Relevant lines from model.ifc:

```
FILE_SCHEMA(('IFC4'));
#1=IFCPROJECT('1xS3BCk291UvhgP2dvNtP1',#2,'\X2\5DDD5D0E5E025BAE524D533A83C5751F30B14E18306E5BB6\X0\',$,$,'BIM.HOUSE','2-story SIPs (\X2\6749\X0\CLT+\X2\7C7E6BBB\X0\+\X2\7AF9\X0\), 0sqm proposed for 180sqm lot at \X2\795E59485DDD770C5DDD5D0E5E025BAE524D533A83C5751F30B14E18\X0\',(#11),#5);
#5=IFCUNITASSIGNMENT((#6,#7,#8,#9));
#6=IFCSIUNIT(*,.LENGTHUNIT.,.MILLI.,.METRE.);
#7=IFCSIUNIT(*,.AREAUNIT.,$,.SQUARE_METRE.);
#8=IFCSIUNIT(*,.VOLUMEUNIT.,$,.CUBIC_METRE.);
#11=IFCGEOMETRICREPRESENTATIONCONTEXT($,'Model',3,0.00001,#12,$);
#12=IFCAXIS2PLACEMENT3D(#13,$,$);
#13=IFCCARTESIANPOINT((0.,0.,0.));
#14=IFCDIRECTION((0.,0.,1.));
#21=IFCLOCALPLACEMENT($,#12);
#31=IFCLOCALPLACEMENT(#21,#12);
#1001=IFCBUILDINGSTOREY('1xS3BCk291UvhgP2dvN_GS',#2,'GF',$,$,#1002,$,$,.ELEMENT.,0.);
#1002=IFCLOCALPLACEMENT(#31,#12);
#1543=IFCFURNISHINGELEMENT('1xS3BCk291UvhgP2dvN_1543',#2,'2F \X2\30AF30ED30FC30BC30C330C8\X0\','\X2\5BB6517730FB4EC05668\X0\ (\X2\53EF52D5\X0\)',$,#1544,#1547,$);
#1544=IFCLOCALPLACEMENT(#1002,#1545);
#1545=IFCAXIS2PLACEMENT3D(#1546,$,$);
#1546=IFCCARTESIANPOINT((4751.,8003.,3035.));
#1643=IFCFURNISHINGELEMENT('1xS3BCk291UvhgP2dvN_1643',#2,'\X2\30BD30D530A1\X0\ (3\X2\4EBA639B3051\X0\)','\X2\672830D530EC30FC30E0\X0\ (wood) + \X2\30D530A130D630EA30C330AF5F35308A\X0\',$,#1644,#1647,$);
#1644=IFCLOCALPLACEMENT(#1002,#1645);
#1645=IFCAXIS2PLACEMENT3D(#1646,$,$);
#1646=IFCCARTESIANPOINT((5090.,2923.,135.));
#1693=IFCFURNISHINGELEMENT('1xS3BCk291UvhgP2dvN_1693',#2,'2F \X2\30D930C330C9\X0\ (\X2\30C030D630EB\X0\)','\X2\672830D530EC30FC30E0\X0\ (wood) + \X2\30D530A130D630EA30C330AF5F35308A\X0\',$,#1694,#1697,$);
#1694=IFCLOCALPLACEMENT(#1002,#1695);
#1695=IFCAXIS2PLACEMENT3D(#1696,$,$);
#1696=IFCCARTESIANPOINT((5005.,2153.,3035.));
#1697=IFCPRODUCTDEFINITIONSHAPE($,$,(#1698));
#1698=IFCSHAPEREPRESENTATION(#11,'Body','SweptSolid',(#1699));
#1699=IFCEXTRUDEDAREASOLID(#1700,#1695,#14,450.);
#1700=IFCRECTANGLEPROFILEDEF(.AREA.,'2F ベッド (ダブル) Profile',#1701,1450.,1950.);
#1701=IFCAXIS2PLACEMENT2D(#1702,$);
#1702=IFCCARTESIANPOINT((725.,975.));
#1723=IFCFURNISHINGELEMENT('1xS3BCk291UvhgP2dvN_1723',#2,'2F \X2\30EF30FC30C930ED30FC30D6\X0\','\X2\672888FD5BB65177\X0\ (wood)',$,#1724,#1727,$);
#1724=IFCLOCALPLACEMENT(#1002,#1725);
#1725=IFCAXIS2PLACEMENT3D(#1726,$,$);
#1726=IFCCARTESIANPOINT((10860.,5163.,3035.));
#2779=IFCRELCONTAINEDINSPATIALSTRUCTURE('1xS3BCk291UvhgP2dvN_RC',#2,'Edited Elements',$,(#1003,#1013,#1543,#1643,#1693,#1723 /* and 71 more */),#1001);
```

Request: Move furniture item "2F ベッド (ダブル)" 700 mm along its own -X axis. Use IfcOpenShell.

```python
import ifcopenshell
import ifcopenshell.api.geometry
import ifcopenshell.util.placement
import ifcopenshell.util.unit

model = ifcopenshell.open("model.ifc")
unit_scale = ifcopenshell.util.unit.calculate_unit_scale(model)

item = model.by_guid("1xS3BCk291UvhgP2dvN_1693")
matrix = ifcopenshell.util.placement.get_local_placement(item.ObjectPlacement)
matrix[:3, 3] -= matrix[:3, 0] * 0.7 / unit_scale
ifcopenshell.api.geometry.edit_object_placement(model, product=item, matrix=matrix, is_si=False)

print(ifcopenshell.util.placement.get_local_placement(item.ObjectPlacement).round(3) + 0.0)

model.write("model_v2.ifc")
```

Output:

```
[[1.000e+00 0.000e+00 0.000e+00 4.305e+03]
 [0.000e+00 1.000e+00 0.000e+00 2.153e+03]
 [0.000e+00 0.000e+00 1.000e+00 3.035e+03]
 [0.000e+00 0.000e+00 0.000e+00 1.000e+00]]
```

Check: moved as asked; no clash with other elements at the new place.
